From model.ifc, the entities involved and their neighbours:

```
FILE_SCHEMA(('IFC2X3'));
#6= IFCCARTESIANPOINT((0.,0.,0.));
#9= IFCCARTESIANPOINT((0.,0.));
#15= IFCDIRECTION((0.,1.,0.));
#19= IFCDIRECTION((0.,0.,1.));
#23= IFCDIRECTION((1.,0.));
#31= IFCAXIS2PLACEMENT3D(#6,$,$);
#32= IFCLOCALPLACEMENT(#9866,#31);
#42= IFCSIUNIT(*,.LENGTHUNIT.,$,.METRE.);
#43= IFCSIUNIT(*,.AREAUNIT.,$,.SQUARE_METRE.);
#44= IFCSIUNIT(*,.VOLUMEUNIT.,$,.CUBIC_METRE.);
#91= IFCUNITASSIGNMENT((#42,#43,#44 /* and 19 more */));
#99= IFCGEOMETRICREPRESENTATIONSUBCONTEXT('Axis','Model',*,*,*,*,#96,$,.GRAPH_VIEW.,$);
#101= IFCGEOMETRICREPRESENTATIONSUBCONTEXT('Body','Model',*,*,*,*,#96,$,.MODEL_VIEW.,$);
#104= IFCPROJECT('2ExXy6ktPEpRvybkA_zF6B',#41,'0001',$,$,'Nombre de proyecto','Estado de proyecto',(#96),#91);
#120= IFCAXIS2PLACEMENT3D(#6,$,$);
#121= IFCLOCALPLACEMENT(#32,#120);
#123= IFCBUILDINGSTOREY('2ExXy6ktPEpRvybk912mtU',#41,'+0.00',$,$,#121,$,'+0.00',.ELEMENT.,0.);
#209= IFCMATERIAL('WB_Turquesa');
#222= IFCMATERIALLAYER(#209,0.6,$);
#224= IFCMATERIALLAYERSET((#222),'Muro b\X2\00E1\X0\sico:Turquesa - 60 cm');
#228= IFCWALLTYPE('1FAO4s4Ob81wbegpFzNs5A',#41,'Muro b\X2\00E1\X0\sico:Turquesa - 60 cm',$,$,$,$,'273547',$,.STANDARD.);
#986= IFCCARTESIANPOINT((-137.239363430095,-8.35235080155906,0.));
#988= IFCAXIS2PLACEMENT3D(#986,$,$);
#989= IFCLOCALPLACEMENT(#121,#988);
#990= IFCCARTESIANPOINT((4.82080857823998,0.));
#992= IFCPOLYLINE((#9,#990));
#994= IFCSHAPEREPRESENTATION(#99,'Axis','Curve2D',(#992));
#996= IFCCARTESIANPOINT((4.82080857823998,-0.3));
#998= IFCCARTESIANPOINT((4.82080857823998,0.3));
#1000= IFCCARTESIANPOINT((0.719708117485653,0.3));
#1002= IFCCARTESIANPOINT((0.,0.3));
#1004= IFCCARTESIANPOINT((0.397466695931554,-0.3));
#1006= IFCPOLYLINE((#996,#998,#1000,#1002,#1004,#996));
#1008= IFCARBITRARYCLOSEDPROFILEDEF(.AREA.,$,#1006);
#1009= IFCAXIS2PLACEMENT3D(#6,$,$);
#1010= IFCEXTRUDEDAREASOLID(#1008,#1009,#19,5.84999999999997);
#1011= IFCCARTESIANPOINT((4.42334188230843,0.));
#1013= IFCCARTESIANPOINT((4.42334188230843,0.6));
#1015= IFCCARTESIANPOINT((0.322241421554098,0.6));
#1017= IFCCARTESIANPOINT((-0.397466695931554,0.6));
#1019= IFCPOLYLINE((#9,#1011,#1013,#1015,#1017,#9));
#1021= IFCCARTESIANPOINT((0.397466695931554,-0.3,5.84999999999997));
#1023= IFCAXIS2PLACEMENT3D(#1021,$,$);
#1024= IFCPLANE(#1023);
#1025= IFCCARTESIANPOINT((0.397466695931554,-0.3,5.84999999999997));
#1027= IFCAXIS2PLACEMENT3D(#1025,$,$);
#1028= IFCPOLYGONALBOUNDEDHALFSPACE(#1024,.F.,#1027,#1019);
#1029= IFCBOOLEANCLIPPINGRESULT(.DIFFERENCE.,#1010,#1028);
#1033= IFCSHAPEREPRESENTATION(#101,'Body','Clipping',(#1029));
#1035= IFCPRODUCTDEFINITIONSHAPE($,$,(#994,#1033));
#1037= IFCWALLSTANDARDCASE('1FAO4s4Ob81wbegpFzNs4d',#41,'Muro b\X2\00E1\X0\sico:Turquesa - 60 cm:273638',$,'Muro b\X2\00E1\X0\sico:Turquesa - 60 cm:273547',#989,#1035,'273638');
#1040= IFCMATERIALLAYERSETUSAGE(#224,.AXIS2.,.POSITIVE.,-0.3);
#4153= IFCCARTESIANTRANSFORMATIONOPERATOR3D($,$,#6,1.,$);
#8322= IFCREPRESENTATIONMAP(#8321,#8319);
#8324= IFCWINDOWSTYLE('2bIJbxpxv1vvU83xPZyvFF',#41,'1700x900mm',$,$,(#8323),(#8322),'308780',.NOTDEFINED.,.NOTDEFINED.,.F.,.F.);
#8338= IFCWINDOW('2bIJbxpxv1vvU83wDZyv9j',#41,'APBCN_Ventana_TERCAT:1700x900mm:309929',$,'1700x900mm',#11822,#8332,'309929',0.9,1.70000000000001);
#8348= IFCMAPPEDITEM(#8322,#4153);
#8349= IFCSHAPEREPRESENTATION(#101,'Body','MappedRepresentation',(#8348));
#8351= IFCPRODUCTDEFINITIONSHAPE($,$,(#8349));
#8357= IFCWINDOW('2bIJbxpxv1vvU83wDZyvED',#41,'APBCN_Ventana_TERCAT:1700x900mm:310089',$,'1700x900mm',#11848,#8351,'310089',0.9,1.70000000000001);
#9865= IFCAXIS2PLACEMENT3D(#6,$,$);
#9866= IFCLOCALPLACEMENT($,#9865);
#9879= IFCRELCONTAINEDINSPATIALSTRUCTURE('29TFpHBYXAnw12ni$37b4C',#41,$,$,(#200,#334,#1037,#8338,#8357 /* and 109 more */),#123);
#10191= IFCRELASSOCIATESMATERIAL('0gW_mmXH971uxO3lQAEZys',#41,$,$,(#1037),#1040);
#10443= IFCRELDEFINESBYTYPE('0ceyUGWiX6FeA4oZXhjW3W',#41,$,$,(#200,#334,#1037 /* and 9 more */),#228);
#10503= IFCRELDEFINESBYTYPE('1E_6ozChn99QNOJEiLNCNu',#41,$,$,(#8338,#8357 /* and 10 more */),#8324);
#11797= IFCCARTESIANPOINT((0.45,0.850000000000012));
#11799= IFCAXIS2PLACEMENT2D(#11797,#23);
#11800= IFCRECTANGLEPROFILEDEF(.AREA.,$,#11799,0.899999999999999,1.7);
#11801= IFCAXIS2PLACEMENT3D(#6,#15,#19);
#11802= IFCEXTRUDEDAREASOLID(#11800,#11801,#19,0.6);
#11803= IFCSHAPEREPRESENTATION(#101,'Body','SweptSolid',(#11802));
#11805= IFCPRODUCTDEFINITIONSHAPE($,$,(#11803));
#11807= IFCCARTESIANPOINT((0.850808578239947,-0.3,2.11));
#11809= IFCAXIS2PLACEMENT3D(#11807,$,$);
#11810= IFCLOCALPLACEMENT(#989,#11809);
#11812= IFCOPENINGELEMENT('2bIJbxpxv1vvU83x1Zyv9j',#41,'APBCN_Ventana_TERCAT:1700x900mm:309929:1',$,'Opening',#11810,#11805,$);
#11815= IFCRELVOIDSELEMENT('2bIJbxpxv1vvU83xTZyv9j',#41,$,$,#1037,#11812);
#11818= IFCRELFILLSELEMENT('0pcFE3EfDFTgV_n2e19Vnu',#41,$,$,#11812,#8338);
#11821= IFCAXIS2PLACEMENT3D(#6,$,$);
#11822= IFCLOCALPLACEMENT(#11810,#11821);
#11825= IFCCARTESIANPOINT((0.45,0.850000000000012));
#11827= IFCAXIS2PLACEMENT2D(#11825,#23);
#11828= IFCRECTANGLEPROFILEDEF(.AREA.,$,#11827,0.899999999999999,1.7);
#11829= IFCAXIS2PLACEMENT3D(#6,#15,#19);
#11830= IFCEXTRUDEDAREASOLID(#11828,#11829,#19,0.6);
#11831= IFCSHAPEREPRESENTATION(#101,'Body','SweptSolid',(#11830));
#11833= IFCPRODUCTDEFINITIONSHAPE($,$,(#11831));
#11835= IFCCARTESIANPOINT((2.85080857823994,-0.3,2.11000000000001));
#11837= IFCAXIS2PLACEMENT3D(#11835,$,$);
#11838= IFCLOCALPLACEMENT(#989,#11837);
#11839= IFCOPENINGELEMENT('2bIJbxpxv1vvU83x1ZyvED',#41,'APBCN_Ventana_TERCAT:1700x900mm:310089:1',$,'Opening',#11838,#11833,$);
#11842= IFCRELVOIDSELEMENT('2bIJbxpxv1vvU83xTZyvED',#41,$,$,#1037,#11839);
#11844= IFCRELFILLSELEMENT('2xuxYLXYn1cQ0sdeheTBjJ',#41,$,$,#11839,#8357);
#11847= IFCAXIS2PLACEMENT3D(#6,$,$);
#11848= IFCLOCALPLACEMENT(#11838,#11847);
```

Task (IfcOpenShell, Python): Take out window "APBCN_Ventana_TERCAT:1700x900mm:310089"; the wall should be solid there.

```python
import ifcopenshell
import ifcopenshell.api.feature
import ifcopenshell.api.root
import ifcopenshell.geom
import ifcopenshell.util.shape

model = ifcopenshell.open("model.ifc")
settings = ifcopenshell.geom.settings()


def volume(element):
    """Net volume in cubic metres, openings subtracted."""
    shape = ifcopenshell.geom.create_shape(settings, element)
    return ifcopenshell.util.shape.get_volume(shape.geometry)


window = model.by_guid("2bIJbxpxv1vvU83wDZyvED")
opening = window.FillsVoids[0].RelatingOpeningElement
wall = opening.VoidsElements[0].RelatingBuildingElement
before = volume(wall)

ifcopenshell.api.root.remove_product(model, product=window)
ifcopenshell.api.feature.remove_feature(model, feature=opening)

after = volume(wall)

print(f"wall volume {before:.3f} -> {after:.3f} m3")

model.write("model_edited.ifc")
```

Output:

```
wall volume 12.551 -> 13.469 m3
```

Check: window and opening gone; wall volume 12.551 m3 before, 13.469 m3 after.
